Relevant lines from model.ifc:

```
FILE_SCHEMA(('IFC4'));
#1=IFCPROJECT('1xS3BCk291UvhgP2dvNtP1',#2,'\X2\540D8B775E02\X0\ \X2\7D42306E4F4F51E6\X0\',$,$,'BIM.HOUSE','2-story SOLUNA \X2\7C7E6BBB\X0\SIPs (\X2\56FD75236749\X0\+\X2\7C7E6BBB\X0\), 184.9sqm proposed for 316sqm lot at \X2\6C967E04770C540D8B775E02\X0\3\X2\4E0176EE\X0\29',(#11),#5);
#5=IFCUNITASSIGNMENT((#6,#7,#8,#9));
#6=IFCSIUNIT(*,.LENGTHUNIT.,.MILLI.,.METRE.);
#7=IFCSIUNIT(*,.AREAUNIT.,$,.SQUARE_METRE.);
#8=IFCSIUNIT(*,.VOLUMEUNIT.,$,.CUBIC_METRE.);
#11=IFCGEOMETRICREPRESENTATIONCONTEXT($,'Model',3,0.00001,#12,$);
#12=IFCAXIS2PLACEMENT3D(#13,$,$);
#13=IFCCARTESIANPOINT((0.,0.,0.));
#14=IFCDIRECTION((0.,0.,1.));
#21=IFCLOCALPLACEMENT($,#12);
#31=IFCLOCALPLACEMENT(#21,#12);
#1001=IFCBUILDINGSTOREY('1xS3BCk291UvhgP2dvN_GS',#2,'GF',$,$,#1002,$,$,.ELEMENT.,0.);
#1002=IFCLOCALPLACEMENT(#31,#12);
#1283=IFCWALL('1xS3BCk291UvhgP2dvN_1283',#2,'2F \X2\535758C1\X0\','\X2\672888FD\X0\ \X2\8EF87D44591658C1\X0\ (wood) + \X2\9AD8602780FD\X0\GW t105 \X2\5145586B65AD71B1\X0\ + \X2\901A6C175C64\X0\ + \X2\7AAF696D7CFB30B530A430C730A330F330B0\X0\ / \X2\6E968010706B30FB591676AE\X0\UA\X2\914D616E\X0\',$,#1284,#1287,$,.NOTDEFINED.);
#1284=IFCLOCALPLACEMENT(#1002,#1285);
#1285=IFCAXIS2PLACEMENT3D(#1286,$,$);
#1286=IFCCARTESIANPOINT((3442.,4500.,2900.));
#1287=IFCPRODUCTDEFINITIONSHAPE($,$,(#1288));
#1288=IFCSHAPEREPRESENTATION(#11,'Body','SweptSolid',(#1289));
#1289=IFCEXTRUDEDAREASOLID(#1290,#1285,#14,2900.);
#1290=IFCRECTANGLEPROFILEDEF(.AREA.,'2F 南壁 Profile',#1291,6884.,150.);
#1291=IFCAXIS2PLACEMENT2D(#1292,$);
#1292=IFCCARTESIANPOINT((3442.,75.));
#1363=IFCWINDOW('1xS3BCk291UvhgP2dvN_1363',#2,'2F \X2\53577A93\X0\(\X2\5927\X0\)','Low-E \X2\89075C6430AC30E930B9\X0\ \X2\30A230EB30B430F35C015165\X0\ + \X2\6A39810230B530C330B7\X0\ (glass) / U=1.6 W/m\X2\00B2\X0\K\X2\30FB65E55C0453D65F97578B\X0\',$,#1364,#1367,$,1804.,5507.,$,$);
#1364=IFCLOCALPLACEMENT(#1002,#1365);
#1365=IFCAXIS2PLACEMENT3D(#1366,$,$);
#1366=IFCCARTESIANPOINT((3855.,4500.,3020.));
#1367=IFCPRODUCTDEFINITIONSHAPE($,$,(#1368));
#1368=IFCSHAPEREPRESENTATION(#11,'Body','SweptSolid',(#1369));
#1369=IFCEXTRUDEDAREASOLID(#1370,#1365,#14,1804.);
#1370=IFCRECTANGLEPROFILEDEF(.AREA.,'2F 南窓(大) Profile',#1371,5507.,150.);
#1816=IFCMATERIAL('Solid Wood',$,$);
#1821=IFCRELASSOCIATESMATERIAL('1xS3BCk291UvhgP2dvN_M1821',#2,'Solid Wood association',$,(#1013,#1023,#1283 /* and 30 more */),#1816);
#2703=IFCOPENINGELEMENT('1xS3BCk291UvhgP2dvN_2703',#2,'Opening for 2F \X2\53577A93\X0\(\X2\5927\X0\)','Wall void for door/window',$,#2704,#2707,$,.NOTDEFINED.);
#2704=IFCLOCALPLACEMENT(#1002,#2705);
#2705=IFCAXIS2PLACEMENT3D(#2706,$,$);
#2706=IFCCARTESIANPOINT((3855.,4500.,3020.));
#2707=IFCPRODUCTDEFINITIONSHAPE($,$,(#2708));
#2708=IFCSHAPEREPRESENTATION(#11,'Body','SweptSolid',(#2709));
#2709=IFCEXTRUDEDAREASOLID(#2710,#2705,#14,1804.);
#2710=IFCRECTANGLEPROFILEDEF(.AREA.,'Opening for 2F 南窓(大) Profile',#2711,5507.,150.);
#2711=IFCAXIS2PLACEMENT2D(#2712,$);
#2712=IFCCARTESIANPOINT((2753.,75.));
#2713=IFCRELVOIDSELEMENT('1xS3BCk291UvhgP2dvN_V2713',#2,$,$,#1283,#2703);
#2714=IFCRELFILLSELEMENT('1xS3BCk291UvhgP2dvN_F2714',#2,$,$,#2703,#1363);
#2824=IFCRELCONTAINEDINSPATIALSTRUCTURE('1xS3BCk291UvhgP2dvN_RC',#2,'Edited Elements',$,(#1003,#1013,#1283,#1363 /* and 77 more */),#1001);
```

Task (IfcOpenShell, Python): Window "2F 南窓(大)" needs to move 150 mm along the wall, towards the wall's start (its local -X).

```python
import ifcopenshell
import ifcopenshell.api.geometry
import ifcopenshell.util.placement

model = ifcopenshell.open("model.ifc")

window = model.by_guid("1xS3BCk291UvhgP2dvN_1363")
opening = window.FillsVoids[0].RelatingOpeningElement
wall = opening.VoidsElements[0].RelatingBuildingElement

wall_matrix = ifcopenshell.util.placement.get_local_placement(wall.ObjectPlacement)
shift = wall_matrix[:3, 0] * -150.0
before = ifcopenshell.util.placement.get_local_placement(window.ObjectPlacement)[:3, 3].copy()

# The window is not placed relative to its opening, so move both.
for product in (opening, window):
    matrix = ifcopenshell.util.placement.get_local_placement(product.ObjectPlacement)
    matrix[:3, 3] += shift
    ifcopenshell.api.geometry.edit_object_placement(model, product=product, matrix=matrix, is_si=False)

after = ifcopenshell.util.placement.get_local_placement(window.ObjectPlacement)[:3, 3]
print("window moved by", (after - before).round(3) + 0.0)

model.write("model_edited.ifc")
```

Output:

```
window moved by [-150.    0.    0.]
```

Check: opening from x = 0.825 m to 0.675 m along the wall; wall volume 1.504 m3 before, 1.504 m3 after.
